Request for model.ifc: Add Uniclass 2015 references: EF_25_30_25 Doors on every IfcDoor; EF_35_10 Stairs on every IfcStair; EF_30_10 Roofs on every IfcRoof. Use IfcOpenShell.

First a look at what the model holds.

```python
import ifcopenshell

model = ifcopenshell.open("model.ifc")
print(model.schema)
print("classifications:", [c.Name for c in model.by_type("IfcClassification")])
for ifc_class in ("IfcDoor", "IfcRoof", "IfcStair", "IfcWall", "IfcWindow"):
    print(ifc_class, len(model.by_type(ifc_class)))
```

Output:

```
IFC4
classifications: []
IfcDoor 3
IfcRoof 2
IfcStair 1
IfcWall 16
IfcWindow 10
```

```python
import ifcopenshell
import ifcopenshell.api.classification

model = ifcopenshell.open("model.ifc")

system = ifcopenshell.api.classification.add_classification(model, classification="Uniclass 2015")

codes = {
    "IfcDoor": ("EF_25_30_25", "Doors"),
    "IfcStair": ("EF_35_10", "Stairs"),
    "IfcRoof": ("EF_30_10", "Roofs"),
}
for ifc_class, (code, name) in codes.items():
    products = model.by_type(ifc_class)
    ifcopenshell.api.classification.add_reference(
        model, products=products, classification=system, identification=code, name=name
    )
    print(code, len(products))

model.write("model_rev.ifc")
```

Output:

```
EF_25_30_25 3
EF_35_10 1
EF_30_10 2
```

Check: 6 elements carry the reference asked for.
